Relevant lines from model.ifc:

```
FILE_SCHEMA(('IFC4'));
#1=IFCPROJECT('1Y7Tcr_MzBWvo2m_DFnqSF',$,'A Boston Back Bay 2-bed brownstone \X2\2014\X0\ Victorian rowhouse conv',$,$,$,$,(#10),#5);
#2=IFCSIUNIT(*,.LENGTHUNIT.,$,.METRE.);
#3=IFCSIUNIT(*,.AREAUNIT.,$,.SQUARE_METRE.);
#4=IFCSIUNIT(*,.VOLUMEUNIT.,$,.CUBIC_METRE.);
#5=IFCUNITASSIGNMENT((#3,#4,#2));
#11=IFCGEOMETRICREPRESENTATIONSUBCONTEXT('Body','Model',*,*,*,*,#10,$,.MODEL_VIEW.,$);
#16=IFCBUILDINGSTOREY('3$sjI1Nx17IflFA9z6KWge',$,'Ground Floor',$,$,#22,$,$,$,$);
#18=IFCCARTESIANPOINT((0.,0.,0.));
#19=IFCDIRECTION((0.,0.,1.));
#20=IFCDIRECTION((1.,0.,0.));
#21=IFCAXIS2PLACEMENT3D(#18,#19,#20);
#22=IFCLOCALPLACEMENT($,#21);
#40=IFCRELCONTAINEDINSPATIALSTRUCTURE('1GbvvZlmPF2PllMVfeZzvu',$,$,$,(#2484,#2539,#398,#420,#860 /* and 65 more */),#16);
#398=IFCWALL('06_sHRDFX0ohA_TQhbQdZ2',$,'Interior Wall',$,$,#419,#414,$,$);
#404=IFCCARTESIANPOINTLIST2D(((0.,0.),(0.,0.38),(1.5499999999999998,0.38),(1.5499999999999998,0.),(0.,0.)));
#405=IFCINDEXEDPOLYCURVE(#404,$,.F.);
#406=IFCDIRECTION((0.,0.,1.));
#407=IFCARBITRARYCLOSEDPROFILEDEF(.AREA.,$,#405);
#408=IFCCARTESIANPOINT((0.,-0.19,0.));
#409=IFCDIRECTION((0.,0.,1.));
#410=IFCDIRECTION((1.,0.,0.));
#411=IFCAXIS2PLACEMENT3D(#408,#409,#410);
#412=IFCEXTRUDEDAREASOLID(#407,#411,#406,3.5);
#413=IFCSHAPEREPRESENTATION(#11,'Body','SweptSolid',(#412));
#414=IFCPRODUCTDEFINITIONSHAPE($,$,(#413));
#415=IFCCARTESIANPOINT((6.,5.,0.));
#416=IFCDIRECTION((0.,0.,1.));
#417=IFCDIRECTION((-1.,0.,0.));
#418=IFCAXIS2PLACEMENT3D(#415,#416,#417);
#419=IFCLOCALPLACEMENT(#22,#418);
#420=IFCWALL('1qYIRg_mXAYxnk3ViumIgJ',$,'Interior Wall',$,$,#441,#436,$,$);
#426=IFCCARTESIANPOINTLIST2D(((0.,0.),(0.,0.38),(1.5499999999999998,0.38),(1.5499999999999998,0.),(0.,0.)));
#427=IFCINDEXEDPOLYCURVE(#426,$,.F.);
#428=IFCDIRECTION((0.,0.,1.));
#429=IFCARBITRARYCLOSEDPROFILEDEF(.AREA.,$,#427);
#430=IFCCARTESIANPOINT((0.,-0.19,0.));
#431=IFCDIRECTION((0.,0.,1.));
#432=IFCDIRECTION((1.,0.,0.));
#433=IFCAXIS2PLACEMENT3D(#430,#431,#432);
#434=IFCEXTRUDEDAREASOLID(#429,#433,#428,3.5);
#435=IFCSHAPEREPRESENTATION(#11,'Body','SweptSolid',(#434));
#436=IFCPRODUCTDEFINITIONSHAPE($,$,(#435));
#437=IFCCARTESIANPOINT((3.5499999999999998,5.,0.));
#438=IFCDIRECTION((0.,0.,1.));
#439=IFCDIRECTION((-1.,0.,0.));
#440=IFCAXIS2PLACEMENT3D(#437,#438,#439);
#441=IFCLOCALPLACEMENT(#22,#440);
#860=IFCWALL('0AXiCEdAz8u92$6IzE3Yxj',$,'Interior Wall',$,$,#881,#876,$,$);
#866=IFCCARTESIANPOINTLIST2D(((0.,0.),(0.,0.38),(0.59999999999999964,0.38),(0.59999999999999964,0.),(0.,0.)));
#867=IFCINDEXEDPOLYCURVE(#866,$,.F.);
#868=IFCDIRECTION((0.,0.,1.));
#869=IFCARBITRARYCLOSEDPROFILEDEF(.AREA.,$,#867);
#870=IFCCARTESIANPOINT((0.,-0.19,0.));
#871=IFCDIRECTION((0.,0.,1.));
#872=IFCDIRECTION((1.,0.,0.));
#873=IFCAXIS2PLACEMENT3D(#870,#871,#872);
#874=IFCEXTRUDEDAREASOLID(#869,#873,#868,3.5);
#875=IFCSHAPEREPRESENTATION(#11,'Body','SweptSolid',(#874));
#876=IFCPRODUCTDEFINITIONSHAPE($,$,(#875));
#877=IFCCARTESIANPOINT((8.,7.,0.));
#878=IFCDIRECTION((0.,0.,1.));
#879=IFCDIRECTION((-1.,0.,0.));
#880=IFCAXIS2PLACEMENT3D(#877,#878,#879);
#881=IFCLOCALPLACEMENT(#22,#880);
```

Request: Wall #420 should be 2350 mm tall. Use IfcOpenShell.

```python
import ifcopenshell
import ifcopenshell.geom
import ifcopenshell.util.representation
import ifcopenshell.util.shape

model = ifcopenshell.open("model.ifc")
settings = ifcopenshell.geom.settings()


def volume(element):
    """Net volume in cubic metres, openings subtracted."""
    shape = ifcopenshell.geom.create_shape(settings, element)
    return ifcopenshell.util.shape.get_volume(shape.geometry)


wall = model.by_id(420)
before = volume(wall)

body = ifcopenshell.util.representation.get_representation(wall, "Model", "Body")
solid = body.Items[0]
old_height = solid.Depth
solid.Depth = 2.35
after = volume(wall)

print(f"height {old_height:g} -> {solid.Depth:g}, volume {before:.3f} -> {after:.3f} m3")

model.write("model_v2.ifc")
```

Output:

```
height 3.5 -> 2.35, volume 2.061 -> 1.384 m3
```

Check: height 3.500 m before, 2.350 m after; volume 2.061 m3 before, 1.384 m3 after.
